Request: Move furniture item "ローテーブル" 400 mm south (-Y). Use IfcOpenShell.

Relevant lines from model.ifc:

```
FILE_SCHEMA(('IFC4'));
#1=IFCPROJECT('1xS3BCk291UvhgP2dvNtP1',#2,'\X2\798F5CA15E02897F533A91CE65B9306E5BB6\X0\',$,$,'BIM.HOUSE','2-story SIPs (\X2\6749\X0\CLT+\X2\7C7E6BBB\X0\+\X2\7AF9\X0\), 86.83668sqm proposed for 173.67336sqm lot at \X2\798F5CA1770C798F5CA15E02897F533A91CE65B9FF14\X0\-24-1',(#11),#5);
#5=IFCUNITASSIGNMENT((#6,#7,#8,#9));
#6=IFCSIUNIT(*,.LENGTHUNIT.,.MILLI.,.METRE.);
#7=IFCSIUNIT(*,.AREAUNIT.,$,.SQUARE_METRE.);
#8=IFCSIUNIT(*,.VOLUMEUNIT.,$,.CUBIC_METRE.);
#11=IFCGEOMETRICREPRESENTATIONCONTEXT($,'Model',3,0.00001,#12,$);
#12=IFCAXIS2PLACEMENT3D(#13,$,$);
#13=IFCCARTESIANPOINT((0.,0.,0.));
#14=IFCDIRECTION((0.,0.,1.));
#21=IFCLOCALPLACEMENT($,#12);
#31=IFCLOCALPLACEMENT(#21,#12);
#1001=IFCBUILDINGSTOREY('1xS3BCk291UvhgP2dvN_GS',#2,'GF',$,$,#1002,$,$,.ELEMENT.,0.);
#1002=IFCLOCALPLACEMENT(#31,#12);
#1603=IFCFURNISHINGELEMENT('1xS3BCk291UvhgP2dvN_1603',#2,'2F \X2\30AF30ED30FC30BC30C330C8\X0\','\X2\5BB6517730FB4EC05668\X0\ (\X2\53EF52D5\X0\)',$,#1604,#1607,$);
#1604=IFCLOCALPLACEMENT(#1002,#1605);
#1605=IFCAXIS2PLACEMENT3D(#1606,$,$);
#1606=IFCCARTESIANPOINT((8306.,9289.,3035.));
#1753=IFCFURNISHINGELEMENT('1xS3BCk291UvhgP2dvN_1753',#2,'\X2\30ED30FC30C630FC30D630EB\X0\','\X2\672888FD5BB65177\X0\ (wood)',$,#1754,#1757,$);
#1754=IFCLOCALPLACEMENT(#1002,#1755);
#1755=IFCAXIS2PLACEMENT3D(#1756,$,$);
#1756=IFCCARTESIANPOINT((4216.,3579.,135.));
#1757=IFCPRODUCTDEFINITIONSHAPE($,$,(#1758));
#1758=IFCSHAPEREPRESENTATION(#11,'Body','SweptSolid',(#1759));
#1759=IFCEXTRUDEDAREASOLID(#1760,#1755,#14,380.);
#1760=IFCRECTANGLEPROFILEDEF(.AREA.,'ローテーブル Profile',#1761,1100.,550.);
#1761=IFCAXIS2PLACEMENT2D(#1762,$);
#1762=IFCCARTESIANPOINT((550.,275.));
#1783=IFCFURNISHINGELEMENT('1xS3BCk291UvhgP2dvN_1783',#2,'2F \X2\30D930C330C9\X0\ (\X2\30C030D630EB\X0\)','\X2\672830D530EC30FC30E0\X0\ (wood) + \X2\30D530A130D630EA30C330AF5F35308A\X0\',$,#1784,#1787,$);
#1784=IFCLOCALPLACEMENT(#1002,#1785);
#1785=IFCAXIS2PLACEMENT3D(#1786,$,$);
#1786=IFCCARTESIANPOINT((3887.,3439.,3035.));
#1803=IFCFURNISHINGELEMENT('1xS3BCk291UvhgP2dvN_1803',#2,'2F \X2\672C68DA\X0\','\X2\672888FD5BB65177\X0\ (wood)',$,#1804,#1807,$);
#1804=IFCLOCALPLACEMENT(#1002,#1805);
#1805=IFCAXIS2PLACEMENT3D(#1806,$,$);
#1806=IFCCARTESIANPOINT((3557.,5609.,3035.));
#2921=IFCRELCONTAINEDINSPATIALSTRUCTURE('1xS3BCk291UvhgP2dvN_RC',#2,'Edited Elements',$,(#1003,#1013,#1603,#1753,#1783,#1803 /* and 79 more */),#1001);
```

```python
import ifcopenshell
import ifcopenshell.api.geometry
import ifcopenshell.util.placement
import ifcopenshell.util.unit

model = ifcopenshell.open("model.ifc")
unit_scale = ifcopenshell.util.unit.calculate_unit_scale(model)

item = model.by_id(1753)
matrix = ifcopenshell.util.placement.get_local_placement(item.ObjectPlacement)
matrix[1, 3] -= 0.4 / unit_scale
ifcopenshell.api.geometry.edit_object_placement(model, product=item, matrix=matrix, is_si=False)

print(ifcopenshell.util.placement.get_local_placement(item.ObjectPlacement).round(3) + 0.0)

model.write("model_v2.ifc")
```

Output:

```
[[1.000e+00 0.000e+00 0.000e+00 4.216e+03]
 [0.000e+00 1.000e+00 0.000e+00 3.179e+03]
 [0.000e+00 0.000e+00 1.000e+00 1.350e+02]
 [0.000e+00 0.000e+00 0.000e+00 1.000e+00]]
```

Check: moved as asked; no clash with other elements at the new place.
